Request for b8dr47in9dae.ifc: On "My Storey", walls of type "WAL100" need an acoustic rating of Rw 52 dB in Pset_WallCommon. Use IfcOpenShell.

First a look at what the model holds.

```python
import ifcopenshell
import ifcopenshell.util.element

model = ifcopenshell.open("b8dr47in9dae.ifc")
print(model.schema)
storey = next(s for s in model.by_type("IfcBuildingStorey") if s.Name == "My Storey")
walls = [e for e in ifcopenshell.util.element.get_decomposition(storey) if e.is_a("IfcWall")]
seen = {}
for e in walls:
    element_type = ifcopenshell.util.element.get_type(e)
    key = (element_type.Name if element_type != e and element_type else None, ifcopenshell.util.element.get_pset(e, "Pset_WallCommon", "AcousticRating"))
    seen[key] = seen.get(key, 0) + 1
for (name, value), count in sorted(seen.items(), key=str):
    print(count, "x", name, "|", value)
```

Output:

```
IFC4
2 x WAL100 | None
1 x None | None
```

```python
import ifcopenshell
import ifcopenshell.api.pset
import ifcopenshell.util.element

model = ifcopenshell.open("b8dr47in9dae.ifc")

storey = next(s for s in model.by_type("IfcBuildingStorey") if s.Name == "My Storey")
walls = [e for e in ifcopenshell.util.element.get_decomposition(storey) if e.is_a("IfcWall")]

count = 0
for e in walls:
    element_type = ifcopenshell.util.element.get_type(e)
    if element_type in (None, e) or element_type.Name != "WAL100":
        continue
    # add_pset returns the element's existing set when there is one.
    pset = ifcopenshell.api.pset.add_pset(model, product=e, name="Pset_WallCommon")
    ifcopenshell.api.pset.edit_pset(model, pset=pset, properties={"AcousticRating": "Rw 52 dB"})
    count += 1

print(count, "walls updated")

model.write("b8dr47in9dae_v2.ifc")
```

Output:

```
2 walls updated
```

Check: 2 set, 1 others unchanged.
